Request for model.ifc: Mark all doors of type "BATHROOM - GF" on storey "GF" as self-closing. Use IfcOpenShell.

First a look at what the model holds.

```python
import ifcopenshell
import ifcopenshell.util.element

model = ifcopenshell.open("model.ifc")
print(model.schema)
storey = next(s for s in model.by_type("IfcBuildingStorey") if s.Name == "GF")
doors = [e for e in ifcopenshell.util.element.get_decomposition(storey) if e.is_a("IfcDoor")]
seen = {}
for e in doors:
    element_type = ifcopenshell.util.element.get_type(e)
    key = (element_type.Name if element_type != e and element_type else None, ifcopenshell.util.element.get_pset(e, "Pset_DoorCommon", "SelfClosing"))
    seen[key] = seen.get(key, 0) + 1
for (name, value), count in sorted(seen.items(), key=str):
    print(count, "x", name, "|", value)
```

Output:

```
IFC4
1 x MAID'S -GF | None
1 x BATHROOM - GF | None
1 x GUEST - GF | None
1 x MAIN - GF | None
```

```python
import ifcopenshell
import ifcopenshell.api.pset
import ifcopenshell.util.element

model = ifcopenshell.open("model.ifc")

storey = next(s for s in model.by_type("IfcBuildingStorey") if s.Name == "GF")
doors = [e for e in ifcopenshell.util.element.get_decomposition(storey) if e.is_a("IfcDoor")]

count = 0
for e in doors:
    element_type = ifcopenshell.util.element.get_type(e)
    if element_type in (None, e) or element_type.Name != "BATHROOM - GF":
        continue
    # add_pset returns the element's existing set when there is one.
    pset = ifcopenshell.api.pset.add_pset(model, product=e, name="Pset_DoorCommon")
    ifcopenshell.api.pset.edit_pset(model, pset=pset, properties={"SelfClosing": True})
    count += 1

print(count, "doors updated")

model.write("model-out.ifc")
```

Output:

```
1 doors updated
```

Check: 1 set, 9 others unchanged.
